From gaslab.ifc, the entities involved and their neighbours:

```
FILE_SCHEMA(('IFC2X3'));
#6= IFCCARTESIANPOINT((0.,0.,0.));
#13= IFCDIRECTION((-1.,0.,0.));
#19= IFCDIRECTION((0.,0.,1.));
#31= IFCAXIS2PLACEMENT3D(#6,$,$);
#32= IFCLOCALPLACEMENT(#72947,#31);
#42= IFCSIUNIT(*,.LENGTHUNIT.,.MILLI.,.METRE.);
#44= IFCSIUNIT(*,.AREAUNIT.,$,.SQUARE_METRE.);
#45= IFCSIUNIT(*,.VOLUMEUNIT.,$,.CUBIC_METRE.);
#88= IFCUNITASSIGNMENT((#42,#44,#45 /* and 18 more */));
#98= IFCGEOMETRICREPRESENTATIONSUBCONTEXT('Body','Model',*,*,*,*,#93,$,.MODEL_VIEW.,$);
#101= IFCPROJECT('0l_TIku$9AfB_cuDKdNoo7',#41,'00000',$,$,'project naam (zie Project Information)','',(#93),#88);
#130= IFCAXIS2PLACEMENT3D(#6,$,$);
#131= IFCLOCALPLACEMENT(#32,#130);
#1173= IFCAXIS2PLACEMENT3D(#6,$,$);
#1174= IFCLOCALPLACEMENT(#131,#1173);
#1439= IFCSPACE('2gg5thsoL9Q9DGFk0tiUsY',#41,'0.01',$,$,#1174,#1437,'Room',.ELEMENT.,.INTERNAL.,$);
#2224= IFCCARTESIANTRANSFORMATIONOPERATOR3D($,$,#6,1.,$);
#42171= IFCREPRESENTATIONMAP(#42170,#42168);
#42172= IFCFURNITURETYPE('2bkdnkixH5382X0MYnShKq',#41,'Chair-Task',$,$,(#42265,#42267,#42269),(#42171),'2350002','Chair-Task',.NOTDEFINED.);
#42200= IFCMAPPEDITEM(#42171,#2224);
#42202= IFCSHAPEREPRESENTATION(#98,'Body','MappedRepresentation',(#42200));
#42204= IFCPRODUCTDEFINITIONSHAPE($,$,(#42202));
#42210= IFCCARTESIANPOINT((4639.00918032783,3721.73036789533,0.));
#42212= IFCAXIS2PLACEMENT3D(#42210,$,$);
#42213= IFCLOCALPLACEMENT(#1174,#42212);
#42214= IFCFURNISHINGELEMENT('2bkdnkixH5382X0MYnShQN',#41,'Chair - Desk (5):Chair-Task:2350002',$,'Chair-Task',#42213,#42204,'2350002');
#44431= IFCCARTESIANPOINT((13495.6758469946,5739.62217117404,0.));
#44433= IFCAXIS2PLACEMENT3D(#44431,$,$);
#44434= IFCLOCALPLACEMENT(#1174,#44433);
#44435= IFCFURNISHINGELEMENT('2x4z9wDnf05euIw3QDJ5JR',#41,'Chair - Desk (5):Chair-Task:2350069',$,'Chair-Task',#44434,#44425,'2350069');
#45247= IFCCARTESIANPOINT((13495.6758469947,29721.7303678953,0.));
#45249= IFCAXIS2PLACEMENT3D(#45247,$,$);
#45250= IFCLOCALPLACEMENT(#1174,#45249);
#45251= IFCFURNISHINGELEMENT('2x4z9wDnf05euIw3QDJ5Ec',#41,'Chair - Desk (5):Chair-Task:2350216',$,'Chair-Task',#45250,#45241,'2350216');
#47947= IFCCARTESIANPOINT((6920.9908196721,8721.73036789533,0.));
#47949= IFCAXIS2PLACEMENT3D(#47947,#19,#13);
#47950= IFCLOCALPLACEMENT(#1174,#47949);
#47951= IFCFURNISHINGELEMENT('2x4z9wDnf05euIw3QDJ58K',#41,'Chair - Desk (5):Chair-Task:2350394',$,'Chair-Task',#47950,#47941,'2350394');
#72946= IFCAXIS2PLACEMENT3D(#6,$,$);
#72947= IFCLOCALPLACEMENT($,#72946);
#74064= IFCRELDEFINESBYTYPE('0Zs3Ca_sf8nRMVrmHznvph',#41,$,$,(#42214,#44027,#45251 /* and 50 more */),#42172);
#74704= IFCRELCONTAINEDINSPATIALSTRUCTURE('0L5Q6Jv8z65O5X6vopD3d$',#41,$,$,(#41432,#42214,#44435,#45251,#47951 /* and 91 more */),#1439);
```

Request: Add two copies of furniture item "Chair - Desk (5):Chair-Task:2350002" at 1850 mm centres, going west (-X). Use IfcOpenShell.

```python
import numpy as np
import ifcopenshell
import ifcopenshell.api.geometry
import ifcopenshell.api.root
import ifcopenshell.util.element
import ifcopenshell.util.placement
import ifcopenshell.util.unit

model = ifcopenshell.open("gaslab.ifc")
unit_scale = ifcopenshell.util.unit.calculate_unit_scale(model)


def reuse_history(source, copy):
    """copy_class also copies each property set's owner history, people and application; keep the originals."""
    for rel in copy.IsDefinedBy:
        if rel.is_a("IfcRelDefinesByProperties") and (history := rel.RelatingPropertyDefinition.OwnerHistory):
            rel.RelatingPropertyDefinition.OwnerHistory = source.OwnerHistory
            ifcopenshell.util.element.remove_deep2(model, history)


source = model.by_guid("2bkdnkixH5382X0MYnShQN")
base = ifcopenshell.util.placement.get_local_placement(source.ObjectPlacement)
step = np.array([-1.0, 0.0, 0.0]) * 1.85 / unit_scale

for i in range(1, 3):
    copy = ifcopenshell.api.root.copy_class(model, product=source)
    copy.Representation = ifcopenshell.util.element.copy_deep(
        model, source.Representation, exclude=["IfcGeometricRepresentationContext", "IfcRepresentationMap"]
    )
    copy.Name = "Chair - Desk (5):Chair-Task"
    copy.Tag = None
    reuse_history(source, copy)
    matrix = base.copy()
    matrix[:3, 3] += i * step
    print("added at", matrix[:3, 3].round(3) + 0.0)
    ifcopenshell.api.geometry.edit_object_placement(model, product=copy, matrix=matrix, is_si=False)

model.write("gaslab_edited.ifc")
```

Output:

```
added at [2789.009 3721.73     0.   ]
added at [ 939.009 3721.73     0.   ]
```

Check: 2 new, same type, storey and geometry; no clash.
